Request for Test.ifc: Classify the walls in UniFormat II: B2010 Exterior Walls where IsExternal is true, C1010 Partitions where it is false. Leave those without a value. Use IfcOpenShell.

First a look at what the model holds.

```python
import ifcopenshell
import ifcopenshell.util.element

model = ifcopenshell.open("Test.ifc")
print(model.schema)
print("classifications:", [c.Name for c in model.by_type("IfcClassification")])
values = [ifcopenshell.util.element.get_pset(e, "Pset_WallCommon", "IsExternal") for e in model.by_type("IfcWall")]
for value in (True, False, None):
    print("IsExternal", value, values.count(value))
```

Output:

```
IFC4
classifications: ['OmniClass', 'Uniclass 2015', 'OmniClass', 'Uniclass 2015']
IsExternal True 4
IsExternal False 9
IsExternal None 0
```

```python
import ifcopenshell
import ifcopenshell.api.classification
import ifcopenshell.util.element

model = ifcopenshell.open("Test.ifc")

system = ifcopenshell.api.classification.add_classification(model, classification="UniFormat II")

walls = model.by_type("IfcWall")
external = {e: ifcopenshell.util.element.get_pset(e, "Pset_WallCommon", "IsExternal") for e in walls}
for flag, code, name in ((True, "B2010", "Exterior Walls"), (False, "C1010", "Partitions")):
    products = [e for e in walls if external[e] is flag]
    ifcopenshell.api.classification.add_reference(
        model, products=products, classification=system, identification=code, name=name
    )
    print(code, len(products))

model.write("Test_rev.ifc")
```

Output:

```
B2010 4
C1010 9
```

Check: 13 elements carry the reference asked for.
